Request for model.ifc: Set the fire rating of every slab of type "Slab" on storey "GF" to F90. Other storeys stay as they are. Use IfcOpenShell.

First a look at what the model holds.

```python
import ifcopenshell
import ifcopenshell.util.element

model = ifcopenshell.open("model.ifc")
print(model.schema)
storey = next(s for s in model.by_type("IfcBuildingStorey") if s.Name == "GF")
slabs = [e for e in ifcopenshell.util.element.get_decomposition(storey) if e.is_a("IfcSlab")]
seen = {}
for e in slabs:
    element_type = ifcopenshell.util.element.get_type(e)
    key = (element_type.Name if element_type != e and element_type else None, ifcopenshell.util.element.get_pset(e, "Pset_SlabCommon", "FireRating"))
    seen[key] = seen.get(key, 0) + 1
for (name, value), count in sorted(seen.items(), key=str):
    print(count, "x", name, "|", value)
```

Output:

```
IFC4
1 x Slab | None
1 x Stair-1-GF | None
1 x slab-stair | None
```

```python
import ifcopenshell
import ifcopenshell.api.pset
import ifcopenshell.util.element

model = ifcopenshell.open("model.ifc")

storey = next(s for s in model.by_type("IfcBuildingStorey") if s.Name == "GF")
slabs = [e for e in ifcopenshell.util.element.get_decomposition(storey) if e.is_a("IfcSlab")]

count = 0
for e in slabs:
    element_type = ifcopenshell.util.element.get_type(e)
    if element_type in (None, e) or element_type.Name != "Slab":
        continue
    # add_pset returns the element's existing set when there is one.
    pset = ifcopenshell.api.pset.add_pset(model, product=e, name="Pset_SlabCommon")
    ifcopenshell.api.pset.edit_pset(model, pset=pset, properties={"FireRating": "F90"})
    count += 1

print(count, "slabs updated")

model.write("model-out.ifc")
```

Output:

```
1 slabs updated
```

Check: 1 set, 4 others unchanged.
